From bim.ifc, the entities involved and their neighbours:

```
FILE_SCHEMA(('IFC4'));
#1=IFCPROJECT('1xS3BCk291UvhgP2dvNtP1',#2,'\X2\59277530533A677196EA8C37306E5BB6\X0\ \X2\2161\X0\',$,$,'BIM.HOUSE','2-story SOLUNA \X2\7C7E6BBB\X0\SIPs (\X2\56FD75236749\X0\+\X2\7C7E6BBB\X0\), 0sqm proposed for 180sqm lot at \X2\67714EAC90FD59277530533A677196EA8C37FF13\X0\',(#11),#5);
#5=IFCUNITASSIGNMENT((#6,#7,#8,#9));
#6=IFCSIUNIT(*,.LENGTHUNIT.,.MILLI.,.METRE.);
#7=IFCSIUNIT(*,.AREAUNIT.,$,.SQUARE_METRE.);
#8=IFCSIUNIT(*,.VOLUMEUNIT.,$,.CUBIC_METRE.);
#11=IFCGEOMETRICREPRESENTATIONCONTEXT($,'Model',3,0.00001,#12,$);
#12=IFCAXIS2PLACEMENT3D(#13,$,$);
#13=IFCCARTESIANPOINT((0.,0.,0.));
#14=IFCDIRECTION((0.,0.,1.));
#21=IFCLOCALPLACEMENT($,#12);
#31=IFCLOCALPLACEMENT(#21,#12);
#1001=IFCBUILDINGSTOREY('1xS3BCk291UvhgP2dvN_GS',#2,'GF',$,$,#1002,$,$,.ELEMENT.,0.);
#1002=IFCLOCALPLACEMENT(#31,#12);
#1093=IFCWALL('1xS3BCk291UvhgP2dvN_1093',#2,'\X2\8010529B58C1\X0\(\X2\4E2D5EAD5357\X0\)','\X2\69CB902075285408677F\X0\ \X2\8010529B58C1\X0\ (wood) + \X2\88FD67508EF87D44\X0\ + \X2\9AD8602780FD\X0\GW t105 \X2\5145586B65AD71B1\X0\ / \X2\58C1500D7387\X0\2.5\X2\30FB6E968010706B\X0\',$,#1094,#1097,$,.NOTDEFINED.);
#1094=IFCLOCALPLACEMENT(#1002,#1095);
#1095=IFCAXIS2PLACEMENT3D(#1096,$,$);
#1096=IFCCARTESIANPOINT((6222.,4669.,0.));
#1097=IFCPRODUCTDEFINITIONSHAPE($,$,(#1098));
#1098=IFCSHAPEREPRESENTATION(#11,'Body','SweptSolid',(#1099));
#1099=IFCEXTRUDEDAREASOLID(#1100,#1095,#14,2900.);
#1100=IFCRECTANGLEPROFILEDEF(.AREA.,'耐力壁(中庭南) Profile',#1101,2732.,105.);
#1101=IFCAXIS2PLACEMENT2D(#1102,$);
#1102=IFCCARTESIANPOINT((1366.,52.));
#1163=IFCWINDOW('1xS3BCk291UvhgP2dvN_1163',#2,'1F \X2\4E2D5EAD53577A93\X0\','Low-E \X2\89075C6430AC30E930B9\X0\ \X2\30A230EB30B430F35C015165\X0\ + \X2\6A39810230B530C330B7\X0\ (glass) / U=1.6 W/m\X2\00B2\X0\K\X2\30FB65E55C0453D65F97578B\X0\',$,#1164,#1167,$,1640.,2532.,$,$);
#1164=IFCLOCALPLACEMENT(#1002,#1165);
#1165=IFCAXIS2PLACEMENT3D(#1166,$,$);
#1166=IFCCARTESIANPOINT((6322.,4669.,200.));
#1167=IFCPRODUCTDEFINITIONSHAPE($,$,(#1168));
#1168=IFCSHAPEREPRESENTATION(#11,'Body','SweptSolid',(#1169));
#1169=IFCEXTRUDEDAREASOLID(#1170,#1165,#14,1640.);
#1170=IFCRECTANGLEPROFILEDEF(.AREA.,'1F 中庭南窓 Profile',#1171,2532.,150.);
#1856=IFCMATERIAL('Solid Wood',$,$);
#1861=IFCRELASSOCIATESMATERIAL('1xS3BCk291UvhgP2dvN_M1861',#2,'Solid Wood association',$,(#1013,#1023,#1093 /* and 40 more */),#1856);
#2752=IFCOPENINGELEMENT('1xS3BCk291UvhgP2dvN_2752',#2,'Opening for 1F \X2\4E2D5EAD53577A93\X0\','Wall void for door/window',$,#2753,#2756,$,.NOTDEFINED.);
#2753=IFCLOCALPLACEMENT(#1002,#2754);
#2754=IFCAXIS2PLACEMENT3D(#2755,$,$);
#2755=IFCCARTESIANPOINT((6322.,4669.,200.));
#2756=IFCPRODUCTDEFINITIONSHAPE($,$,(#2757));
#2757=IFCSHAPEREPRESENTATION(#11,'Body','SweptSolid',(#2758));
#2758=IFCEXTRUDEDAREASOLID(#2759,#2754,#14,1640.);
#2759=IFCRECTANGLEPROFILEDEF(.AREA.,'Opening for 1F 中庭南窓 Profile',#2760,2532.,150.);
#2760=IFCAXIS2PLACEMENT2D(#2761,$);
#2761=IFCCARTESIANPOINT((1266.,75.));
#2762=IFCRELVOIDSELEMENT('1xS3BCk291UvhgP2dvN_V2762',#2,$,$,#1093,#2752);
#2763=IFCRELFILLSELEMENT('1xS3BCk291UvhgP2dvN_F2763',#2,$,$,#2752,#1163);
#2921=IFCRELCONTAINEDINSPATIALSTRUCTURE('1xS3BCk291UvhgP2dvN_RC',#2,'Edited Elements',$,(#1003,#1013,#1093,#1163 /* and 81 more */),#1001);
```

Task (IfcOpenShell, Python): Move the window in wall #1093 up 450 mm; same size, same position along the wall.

```python
import numpy as np
import ifcopenshell
import ifcopenshell.api.geometry
import ifcopenshell.util.placement
import ifcopenshell.util.unit

model = ifcopenshell.open("bim.ifc")
unit_scale = ifcopenshell.util.unit.calculate_unit_scale(model)

window = model.by_guid("1xS3BCk291UvhgP2dvN_1163")
opening = window.FillsVoids[0].RelatingOpeningElement
dz = 0.45 / unit_scale

shift = np.array([0.0, 0.0, dz])
# The window is not placed relative to its opening, so move both.
for product in (opening, window):
    matrix = ifcopenshell.util.placement.get_local_placement(product.ObjectPlacement)
    matrix[:3, 3] += shift
    ifcopenshell.api.geometry.edit_object_placement(model, product=product, matrix=matrix, is_si=False)

print(f"moved by {dz * unit_scale:+.3f} m")

model.write("bim_v2.ifc")
```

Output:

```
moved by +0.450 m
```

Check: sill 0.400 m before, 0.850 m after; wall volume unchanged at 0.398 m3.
